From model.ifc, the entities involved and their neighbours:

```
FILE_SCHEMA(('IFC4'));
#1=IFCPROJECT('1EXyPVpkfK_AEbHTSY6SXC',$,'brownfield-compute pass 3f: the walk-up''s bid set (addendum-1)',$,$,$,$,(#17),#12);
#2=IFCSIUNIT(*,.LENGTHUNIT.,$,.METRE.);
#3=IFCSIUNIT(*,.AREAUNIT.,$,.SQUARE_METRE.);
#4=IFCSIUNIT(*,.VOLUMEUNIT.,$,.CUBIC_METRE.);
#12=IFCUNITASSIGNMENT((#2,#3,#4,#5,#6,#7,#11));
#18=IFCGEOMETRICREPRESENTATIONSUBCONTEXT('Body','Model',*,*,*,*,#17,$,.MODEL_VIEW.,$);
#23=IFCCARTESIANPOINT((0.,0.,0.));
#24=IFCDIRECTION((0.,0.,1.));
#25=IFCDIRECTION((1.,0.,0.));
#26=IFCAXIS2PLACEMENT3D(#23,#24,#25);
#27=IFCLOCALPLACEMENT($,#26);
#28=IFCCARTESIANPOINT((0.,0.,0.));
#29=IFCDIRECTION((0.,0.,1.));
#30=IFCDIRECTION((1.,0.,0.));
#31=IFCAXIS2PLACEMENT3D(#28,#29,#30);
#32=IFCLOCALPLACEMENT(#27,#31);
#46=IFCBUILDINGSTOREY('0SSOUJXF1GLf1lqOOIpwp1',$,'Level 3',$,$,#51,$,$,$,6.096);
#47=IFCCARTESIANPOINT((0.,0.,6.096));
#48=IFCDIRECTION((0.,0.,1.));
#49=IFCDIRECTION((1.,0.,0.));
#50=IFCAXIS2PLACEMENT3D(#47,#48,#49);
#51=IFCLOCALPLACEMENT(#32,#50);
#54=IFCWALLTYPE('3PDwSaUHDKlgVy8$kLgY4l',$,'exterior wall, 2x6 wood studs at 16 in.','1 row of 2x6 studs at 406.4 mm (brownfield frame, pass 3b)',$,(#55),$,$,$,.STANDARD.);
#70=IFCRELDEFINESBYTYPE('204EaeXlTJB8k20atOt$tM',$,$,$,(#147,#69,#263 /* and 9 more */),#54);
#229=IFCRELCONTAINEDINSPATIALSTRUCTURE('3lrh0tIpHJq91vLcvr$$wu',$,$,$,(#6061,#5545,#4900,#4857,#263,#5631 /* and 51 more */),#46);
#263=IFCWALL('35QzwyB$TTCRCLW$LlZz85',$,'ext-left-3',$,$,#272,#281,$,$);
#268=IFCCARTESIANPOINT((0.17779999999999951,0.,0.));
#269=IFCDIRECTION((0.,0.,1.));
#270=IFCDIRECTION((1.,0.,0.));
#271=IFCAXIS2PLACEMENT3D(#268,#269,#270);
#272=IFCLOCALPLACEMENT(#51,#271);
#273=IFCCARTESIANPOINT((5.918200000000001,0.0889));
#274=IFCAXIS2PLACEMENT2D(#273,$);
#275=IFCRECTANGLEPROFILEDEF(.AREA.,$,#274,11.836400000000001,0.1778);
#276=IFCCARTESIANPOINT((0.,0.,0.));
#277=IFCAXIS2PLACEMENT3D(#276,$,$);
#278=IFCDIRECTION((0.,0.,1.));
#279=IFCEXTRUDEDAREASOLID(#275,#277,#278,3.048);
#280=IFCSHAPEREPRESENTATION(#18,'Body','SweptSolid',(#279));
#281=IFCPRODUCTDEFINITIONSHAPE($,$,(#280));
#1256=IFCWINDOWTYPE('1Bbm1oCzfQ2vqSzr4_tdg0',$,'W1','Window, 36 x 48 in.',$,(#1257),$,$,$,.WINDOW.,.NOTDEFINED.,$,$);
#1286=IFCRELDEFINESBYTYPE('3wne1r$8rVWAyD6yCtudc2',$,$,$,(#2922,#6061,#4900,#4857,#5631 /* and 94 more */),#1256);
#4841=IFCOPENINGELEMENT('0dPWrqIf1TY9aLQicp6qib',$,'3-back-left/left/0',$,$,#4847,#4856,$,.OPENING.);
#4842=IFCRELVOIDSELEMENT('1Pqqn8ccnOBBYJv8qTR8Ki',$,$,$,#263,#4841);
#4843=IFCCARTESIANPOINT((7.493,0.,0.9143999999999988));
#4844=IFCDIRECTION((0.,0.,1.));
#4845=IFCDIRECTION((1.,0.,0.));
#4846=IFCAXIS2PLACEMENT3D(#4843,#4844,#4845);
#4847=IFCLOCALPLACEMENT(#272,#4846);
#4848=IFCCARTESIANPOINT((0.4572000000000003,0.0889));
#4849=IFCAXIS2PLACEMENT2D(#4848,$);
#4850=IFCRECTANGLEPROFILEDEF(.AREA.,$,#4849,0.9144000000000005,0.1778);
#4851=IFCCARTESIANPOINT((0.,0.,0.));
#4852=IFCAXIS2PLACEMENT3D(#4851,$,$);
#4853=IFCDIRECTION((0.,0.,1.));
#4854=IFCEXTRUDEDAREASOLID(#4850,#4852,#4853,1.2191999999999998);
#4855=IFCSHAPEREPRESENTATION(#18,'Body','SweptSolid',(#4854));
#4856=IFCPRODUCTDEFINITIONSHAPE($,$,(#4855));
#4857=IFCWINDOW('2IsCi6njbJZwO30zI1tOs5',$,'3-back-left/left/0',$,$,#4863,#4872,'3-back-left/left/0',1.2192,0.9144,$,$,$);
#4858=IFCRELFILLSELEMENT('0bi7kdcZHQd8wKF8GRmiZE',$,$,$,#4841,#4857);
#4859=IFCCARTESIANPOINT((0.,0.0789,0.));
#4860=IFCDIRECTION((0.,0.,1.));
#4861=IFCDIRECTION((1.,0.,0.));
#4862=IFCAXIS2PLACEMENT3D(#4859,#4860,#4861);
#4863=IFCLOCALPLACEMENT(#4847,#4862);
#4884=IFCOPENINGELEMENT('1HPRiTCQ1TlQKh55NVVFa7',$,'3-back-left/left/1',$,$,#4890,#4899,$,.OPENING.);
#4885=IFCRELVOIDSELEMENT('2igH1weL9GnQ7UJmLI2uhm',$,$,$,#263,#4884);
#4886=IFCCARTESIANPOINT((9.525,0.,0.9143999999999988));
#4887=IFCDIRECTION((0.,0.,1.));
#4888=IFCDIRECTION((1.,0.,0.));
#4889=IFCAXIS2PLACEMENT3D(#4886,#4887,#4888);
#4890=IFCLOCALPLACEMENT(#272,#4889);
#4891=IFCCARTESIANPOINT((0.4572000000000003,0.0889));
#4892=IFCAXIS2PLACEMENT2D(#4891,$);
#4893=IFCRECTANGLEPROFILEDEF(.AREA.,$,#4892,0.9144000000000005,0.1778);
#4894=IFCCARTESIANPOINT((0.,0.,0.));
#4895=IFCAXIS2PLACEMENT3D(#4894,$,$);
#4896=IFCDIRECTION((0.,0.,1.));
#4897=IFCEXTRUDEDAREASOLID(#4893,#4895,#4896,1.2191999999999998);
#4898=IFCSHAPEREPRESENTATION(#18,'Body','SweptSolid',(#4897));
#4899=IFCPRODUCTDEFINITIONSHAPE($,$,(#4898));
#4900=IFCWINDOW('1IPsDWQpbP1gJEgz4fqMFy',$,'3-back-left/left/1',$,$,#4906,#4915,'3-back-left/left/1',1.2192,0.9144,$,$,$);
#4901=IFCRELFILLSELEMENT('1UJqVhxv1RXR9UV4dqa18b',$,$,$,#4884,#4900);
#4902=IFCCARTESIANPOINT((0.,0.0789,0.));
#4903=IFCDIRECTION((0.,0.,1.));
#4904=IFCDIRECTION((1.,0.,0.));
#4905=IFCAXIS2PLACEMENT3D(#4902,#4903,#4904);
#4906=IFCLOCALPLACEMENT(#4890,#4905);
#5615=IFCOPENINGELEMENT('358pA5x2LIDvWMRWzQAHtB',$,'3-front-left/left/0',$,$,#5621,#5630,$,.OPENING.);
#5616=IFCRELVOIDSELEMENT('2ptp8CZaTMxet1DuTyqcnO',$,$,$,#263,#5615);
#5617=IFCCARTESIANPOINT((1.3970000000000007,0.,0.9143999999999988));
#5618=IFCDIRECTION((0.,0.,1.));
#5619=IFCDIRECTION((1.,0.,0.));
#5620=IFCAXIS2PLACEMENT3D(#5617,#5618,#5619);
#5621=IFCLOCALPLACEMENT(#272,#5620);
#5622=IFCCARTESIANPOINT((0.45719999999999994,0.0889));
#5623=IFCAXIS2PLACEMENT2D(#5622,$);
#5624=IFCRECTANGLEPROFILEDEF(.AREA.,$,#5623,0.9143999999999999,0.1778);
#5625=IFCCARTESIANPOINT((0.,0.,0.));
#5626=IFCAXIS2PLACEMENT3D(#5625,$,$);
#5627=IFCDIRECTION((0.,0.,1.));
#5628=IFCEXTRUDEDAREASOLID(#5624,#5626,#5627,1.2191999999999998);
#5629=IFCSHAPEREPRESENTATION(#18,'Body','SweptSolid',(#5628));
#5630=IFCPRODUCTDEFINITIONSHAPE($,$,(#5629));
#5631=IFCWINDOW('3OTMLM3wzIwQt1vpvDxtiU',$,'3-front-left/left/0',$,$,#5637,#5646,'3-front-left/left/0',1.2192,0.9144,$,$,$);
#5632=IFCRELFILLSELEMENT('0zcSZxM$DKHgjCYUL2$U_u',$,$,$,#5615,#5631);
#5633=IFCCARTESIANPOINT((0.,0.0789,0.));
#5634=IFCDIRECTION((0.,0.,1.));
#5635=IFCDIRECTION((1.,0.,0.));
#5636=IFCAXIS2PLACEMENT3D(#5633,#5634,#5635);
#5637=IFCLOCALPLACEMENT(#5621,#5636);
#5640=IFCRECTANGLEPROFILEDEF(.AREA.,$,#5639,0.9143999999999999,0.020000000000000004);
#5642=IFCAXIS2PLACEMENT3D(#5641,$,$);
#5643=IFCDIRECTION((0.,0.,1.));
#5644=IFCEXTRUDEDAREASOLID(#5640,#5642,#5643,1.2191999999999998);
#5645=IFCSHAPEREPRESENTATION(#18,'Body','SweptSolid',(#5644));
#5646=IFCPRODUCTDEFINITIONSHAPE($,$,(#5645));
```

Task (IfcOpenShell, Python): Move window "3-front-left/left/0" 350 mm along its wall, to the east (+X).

```python
import ifcopenshell
import ifcopenshell.api.geometry
import ifcopenshell.util.placement

model = ifcopenshell.open("model.ifc")

window = model.by_guid("3OTMLM3wzIwQt1vpvDxtiU")
opening = window.FillsVoids[0].RelatingOpeningElement
wall = opening.VoidsElements[0].RelatingBuildingElement

wall_matrix = ifcopenshell.util.placement.get_local_placement(wall.ObjectPlacement)
shift = wall_matrix[:3, 0] * 0.35
before = ifcopenshell.util.placement.get_local_placement(window.ObjectPlacement)[:3, 3].copy()

# The window is placed relative to its opening, so it follows when the opening moves.
matrix = ifcopenshell.util.placement.get_local_placement(opening.ObjectPlacement)
matrix[:3, 3] += shift
ifcopenshell.api.geometry.edit_object_placement(
    model, product=opening, matrix=matrix, is_si=False, should_transform_children=True
)

after = ifcopenshell.util.placement.get_local_placement(window.ObjectPlacement)[:3, 3]
print("window moved by", (after - before).round(3) + 0.0)

model.write("model_updated.ifc")
```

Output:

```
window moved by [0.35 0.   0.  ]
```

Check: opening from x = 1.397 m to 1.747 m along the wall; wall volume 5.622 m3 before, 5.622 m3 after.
